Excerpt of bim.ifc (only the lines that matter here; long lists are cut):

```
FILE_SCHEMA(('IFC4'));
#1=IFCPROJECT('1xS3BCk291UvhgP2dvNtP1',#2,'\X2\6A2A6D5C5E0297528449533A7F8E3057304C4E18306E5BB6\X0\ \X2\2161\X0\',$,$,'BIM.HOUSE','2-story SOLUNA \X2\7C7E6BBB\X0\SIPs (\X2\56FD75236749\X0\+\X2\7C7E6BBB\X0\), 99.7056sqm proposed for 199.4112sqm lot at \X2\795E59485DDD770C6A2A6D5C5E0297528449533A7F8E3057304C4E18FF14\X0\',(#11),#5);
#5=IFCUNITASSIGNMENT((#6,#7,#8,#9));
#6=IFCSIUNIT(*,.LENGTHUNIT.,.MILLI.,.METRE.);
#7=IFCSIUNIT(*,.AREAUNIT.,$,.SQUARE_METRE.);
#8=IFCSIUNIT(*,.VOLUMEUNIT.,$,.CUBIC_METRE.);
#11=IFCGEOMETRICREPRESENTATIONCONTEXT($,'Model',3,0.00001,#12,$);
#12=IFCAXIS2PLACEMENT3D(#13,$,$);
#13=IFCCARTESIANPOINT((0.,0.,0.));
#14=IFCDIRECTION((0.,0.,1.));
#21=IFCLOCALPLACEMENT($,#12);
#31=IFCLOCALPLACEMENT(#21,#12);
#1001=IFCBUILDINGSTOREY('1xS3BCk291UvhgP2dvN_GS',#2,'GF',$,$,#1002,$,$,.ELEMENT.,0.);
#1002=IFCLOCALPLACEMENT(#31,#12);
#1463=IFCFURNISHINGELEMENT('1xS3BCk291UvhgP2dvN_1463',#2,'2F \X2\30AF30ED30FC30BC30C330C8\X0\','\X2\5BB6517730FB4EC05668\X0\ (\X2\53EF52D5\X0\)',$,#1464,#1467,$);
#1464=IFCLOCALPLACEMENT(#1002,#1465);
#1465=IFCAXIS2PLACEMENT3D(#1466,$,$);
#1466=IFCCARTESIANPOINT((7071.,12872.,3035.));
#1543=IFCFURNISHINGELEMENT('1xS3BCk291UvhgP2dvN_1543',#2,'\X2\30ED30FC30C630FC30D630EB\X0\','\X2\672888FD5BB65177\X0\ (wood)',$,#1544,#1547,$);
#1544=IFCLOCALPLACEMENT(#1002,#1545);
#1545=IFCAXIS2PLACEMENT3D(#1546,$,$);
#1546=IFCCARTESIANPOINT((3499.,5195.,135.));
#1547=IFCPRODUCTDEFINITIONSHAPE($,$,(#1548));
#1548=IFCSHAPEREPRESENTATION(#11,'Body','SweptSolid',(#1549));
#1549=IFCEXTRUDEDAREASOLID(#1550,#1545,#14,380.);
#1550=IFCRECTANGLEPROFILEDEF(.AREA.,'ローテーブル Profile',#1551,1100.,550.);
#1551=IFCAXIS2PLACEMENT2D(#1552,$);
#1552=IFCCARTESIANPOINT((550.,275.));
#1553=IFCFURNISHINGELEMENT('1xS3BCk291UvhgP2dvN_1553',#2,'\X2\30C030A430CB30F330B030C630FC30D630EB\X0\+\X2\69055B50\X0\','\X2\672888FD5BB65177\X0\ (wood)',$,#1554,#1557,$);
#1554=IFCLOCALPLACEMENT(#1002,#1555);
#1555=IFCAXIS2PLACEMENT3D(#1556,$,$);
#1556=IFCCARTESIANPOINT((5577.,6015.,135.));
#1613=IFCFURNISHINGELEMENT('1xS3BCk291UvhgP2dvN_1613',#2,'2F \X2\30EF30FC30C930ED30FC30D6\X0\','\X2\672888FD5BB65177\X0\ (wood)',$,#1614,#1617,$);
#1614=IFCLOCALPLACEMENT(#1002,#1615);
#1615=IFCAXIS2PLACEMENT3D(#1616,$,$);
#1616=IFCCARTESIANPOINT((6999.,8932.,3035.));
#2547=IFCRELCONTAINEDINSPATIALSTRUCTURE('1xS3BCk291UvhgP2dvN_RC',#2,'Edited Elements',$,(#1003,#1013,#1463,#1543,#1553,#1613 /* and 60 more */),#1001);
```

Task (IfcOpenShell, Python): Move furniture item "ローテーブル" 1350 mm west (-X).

```python
import ifcopenshell
import ifcopenshell.api.geometry
import ifcopenshell.util.placement

model = ifcopenshell.open("bim.ifc")

item = model.by_id(1543)
matrix = ifcopenshell.util.placement.get_local_placement(item.ObjectPlacement)
matrix[0, 3] -= 1350.0
ifcopenshell.api.geometry.edit_object_placement(model, product=item, matrix=matrix, is_si=False)

print(ifcopenshell.util.placement.get_local_placement(item.ObjectPlacement).round(3) + 0.0)

model.write("bim_edited.ifc")
```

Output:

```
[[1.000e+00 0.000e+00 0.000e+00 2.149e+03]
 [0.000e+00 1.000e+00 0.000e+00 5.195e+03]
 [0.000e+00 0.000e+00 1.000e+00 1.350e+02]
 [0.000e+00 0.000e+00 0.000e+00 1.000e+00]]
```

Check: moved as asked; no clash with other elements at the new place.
